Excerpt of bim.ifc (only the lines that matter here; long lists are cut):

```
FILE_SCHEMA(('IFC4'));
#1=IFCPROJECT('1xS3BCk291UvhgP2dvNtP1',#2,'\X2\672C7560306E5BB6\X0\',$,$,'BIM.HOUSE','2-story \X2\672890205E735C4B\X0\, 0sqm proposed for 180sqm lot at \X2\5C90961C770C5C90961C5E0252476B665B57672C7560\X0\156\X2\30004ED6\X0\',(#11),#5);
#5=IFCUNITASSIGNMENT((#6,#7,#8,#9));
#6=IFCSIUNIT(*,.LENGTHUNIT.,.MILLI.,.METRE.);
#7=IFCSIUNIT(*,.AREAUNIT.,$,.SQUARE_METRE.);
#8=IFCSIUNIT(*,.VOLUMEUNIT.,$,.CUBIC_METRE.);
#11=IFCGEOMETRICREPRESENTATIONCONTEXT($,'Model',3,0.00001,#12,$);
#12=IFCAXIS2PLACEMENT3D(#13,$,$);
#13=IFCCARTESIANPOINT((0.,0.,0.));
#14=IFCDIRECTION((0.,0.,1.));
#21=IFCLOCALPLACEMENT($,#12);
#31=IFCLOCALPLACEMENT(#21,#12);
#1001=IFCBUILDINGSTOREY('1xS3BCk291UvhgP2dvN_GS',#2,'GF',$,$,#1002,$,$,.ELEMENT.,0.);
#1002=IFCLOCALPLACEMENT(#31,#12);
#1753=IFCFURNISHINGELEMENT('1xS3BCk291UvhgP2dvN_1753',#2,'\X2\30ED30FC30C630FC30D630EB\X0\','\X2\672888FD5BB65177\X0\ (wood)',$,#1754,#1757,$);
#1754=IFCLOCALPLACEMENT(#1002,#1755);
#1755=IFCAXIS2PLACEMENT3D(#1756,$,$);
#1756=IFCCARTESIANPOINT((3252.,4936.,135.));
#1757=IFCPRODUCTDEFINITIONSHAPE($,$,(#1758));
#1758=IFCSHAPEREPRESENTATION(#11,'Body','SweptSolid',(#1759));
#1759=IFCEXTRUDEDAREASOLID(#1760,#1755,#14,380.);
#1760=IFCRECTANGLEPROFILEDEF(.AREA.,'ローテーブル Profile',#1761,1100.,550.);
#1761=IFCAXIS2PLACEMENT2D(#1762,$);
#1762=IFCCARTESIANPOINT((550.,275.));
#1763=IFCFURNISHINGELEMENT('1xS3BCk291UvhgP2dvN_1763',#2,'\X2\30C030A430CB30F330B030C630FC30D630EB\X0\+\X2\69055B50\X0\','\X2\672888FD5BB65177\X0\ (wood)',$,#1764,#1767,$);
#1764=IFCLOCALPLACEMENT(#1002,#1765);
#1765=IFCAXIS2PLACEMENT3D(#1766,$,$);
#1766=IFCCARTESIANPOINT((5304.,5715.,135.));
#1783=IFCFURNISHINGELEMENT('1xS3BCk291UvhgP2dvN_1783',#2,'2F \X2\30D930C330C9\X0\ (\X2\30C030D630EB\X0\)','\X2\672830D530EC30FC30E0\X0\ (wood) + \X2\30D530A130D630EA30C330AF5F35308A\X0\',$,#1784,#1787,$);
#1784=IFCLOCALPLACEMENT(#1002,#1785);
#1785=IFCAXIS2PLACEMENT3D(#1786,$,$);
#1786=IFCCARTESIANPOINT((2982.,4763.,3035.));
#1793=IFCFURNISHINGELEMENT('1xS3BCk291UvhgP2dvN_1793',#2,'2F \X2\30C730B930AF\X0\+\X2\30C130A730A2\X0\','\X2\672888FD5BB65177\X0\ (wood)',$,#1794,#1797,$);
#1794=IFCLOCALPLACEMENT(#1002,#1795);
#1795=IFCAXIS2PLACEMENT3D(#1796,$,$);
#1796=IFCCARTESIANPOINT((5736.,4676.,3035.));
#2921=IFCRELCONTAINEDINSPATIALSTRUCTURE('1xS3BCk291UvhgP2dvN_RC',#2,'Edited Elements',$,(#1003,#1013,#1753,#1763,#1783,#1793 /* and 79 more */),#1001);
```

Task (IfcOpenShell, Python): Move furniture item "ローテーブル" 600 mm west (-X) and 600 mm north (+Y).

```python
import ifcopenshell
import ifcopenshell.api.geometry
import ifcopenshell.util.placement
import ifcopenshell.util.unit

model = ifcopenshell.open("bim.ifc")
unit_scale = ifcopenshell.util.unit.calculate_unit_scale(model)

item = model.by_guid("1xS3BCk291UvhgP2dvN_1753")
matrix = ifcopenshell.util.placement.get_local_placement(item.ObjectPlacement)
matrix[0, 3] -= 0.6 / unit_scale
matrix[1, 3] += 0.6 / unit_scale
ifcopenshell.api.geometry.edit_object_placement(model, product=item, matrix=matrix, is_si=False)

print(ifcopenshell.util.placement.get_local_placement(item.ObjectPlacement).round(3) + 0.0)

model.write("bim_edited.ifc")
```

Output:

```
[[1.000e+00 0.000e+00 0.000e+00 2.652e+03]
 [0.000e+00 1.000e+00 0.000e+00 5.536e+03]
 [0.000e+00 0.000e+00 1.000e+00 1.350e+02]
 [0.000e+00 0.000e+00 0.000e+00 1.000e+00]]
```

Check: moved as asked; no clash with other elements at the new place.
